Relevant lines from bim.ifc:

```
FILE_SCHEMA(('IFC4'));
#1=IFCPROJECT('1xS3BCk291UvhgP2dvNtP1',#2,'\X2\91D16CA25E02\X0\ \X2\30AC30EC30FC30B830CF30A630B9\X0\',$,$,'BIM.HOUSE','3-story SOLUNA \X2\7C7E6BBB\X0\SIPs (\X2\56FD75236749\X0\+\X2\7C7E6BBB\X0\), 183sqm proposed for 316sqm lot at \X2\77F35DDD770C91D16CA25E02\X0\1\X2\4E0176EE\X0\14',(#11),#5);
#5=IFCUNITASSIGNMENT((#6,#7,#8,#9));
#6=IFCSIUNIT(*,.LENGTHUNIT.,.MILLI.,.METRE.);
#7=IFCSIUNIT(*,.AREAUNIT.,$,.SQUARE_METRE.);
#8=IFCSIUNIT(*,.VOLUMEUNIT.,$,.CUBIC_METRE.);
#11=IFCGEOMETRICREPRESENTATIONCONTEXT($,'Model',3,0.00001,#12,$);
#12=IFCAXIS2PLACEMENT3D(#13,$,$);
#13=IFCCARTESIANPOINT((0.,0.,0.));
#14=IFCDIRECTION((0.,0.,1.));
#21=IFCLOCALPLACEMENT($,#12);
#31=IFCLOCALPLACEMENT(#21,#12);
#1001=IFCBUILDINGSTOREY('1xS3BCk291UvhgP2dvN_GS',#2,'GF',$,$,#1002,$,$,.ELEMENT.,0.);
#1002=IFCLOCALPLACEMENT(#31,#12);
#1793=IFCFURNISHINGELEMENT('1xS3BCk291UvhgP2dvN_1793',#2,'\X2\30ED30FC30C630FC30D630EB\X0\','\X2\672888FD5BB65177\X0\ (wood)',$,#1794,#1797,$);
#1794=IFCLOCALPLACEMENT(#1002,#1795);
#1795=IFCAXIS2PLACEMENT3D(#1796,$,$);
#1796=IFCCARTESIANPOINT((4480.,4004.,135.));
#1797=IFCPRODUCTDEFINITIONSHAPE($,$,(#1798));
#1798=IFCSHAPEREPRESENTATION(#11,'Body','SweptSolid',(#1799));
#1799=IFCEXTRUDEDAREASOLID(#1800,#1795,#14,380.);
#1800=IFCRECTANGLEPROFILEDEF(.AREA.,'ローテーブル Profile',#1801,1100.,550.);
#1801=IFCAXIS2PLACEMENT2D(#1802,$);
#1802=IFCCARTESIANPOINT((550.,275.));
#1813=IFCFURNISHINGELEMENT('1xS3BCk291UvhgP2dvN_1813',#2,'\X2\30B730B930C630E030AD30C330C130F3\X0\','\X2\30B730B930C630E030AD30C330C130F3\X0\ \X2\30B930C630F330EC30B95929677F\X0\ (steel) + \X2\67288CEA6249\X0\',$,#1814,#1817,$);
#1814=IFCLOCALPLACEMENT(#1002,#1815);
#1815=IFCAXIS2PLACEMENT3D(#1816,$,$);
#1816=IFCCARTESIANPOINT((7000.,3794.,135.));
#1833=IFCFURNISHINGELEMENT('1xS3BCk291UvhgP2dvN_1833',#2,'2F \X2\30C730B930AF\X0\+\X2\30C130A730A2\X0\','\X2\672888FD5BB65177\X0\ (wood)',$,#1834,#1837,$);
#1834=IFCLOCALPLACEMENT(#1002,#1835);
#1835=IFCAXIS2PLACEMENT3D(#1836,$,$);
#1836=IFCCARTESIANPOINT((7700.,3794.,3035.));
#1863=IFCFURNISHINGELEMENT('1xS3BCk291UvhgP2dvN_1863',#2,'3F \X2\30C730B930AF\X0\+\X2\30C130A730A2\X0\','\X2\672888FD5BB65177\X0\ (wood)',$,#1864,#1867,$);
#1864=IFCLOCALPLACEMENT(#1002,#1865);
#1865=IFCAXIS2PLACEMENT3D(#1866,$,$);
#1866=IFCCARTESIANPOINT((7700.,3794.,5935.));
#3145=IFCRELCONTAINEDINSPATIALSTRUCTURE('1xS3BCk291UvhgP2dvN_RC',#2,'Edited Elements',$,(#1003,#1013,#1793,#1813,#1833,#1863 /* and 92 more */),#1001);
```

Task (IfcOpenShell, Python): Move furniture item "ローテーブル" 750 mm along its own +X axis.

```python
import ifcopenshell
import ifcopenshell.api.geometry
import ifcopenshell.util.placement
import ifcopenshell.util.unit

model = ifcopenshell.open("bim.ifc")
unit_scale = ifcopenshell.util.unit.calculate_unit_scale(model)

item = model.by_guid("1xS3BCk291UvhgP2dvN_1793")
matrix = ifcopenshell.util.placement.get_local_placement(item.ObjectPlacement)
matrix[:3, 3] += matrix[:3, 0] * 0.75 / unit_scale
ifcopenshell.api.geometry.edit_object_placement(model, product=item, matrix=matrix, is_si=False)

print(ifcopenshell.util.placement.get_local_placement(item.ObjectPlacement).round(3) + 0.0)

model.write("bim_v2.ifc")
```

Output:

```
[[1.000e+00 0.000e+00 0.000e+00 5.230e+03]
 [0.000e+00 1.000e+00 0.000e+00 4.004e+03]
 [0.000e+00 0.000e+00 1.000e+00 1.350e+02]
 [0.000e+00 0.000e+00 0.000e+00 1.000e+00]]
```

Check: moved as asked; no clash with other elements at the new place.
